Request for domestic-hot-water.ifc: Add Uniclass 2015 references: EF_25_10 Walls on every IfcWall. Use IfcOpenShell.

First a look at what the model holds.

```python
import ifcopenshell

model = ifcopenshell.open("domestic-hot-water.ifc")
print(model.schema)
print("classifications:", [c.Name for c in model.by_type("IfcClassification")])
for ifc_class in ("IfcDoor", "IfcRoof", "IfcStair", "IfcWall", "IfcWindow"):
    print(ifc_class, len(model.by_type(ifc_class)))
```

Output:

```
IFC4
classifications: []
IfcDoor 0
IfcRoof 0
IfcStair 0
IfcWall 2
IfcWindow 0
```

```python
import ifcopenshell
import ifcopenshell.api.classification

model = ifcopenshell.open("domestic-hot-water.ifc")

system = ifcopenshell.api.classification.add_classification(model, classification="Uniclass 2015")

codes = {
    "IfcWall": ("EF_25_10", "Walls"),
}
for ifc_class, (code, name) in codes.items():
    products = model.by_type(ifc_class)
    ifcopenshell.api.classification.add_reference(
        model, products=products, classification=system, identification=code, name=name
    )
    print(code, len(products))

model.write("domestic-hot-water_edited.ifc")
```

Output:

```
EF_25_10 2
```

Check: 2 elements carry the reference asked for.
